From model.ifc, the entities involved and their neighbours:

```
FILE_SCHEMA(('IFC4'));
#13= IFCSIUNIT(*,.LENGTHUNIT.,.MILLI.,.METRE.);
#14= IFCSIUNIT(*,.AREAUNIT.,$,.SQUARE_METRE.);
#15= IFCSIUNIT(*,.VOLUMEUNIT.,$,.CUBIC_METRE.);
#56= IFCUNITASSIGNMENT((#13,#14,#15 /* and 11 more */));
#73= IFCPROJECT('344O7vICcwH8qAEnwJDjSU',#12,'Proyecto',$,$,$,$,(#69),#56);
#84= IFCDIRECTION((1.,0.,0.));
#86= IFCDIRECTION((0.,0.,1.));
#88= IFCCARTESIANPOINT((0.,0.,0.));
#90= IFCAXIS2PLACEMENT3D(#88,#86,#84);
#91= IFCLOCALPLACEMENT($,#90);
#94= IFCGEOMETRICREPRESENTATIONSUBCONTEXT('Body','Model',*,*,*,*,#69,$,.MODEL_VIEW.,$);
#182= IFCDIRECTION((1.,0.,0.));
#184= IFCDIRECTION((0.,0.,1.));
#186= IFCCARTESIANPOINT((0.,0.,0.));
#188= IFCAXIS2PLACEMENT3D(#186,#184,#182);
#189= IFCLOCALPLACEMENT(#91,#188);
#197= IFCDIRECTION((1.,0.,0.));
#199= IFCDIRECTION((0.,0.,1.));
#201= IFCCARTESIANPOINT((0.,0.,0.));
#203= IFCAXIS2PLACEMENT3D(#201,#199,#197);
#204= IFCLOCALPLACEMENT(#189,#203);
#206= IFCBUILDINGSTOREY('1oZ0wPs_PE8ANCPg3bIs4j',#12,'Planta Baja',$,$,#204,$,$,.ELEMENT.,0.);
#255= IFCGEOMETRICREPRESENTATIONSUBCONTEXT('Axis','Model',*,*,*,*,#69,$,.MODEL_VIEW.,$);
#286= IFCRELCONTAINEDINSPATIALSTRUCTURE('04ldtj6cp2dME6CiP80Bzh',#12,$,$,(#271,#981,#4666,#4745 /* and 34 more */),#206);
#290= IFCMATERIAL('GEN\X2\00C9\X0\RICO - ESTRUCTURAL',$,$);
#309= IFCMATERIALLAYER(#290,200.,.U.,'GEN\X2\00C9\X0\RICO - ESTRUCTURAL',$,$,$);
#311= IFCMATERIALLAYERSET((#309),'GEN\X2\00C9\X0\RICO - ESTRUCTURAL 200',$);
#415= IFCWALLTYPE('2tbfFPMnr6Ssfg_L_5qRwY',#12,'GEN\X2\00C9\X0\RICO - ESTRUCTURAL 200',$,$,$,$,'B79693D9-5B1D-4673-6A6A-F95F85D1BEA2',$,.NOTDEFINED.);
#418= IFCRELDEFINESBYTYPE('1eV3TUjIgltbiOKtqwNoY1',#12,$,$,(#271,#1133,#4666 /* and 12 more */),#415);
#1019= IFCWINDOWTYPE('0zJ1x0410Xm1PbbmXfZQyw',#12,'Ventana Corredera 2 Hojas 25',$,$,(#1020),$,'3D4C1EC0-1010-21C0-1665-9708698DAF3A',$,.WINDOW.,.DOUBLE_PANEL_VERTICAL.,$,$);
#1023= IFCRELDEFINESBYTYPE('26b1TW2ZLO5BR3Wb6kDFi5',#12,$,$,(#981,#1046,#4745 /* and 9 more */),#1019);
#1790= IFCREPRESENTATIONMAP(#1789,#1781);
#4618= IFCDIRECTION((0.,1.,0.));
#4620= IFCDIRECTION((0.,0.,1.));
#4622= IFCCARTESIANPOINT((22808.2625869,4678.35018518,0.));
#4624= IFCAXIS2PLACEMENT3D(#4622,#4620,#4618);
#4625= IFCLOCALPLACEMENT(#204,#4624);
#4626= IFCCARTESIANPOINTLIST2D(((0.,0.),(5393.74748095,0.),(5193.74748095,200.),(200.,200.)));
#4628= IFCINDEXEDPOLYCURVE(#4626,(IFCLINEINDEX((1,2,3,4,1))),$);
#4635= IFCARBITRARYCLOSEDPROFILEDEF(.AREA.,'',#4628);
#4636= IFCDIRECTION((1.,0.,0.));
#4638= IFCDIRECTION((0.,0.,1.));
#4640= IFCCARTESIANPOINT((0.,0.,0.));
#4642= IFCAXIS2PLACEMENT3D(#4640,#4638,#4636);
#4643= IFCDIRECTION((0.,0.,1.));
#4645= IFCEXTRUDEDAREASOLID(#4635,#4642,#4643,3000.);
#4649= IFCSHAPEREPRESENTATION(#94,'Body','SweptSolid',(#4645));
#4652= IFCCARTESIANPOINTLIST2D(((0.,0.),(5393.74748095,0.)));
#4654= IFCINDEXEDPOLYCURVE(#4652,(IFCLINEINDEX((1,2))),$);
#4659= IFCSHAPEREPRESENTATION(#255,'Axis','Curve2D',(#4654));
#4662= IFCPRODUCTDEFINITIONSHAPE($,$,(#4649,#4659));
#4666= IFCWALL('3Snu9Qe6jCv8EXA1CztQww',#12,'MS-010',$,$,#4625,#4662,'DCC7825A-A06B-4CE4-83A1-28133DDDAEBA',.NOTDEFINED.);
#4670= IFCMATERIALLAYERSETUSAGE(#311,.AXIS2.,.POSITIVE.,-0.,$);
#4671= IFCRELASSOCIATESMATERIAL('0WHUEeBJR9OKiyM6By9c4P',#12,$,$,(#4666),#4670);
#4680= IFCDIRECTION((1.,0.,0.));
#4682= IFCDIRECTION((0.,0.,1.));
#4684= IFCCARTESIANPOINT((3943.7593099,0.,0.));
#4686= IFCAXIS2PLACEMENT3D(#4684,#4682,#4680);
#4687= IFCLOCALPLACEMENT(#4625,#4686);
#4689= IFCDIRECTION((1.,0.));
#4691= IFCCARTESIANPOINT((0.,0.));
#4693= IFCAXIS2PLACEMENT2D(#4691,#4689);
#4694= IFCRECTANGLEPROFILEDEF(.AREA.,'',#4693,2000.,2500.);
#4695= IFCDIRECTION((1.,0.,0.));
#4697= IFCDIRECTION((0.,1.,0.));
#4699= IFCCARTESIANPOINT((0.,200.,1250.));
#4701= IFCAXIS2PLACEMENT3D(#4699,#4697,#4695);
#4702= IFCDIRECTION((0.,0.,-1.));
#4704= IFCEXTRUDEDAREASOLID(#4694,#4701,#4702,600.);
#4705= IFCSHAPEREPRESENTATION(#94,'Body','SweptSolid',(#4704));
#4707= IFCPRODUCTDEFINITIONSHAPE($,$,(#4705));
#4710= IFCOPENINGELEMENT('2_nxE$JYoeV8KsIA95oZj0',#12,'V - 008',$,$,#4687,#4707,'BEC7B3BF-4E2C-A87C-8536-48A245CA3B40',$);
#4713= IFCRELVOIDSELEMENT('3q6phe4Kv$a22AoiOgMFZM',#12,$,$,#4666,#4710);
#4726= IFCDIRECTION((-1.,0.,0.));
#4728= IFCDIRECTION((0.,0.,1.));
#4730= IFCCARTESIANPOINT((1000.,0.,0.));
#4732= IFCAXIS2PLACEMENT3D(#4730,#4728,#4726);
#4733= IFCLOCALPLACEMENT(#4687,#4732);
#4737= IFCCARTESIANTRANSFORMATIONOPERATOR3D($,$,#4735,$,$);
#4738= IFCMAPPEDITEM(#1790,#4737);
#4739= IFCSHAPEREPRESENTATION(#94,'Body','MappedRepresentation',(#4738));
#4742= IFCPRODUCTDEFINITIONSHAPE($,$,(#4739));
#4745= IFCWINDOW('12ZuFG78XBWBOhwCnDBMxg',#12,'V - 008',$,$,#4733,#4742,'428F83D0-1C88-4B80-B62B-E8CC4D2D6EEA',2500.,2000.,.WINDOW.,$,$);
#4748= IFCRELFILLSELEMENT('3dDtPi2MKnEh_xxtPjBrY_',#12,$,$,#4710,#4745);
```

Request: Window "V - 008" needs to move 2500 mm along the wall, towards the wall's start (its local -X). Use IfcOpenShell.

```python
import ifcopenshell
import ifcopenshell.api.geometry
import ifcopenshell.util.placement

model = ifcopenshell.open("model.ifc")

window = model.by_guid("12ZuFG78XBWBOhwCnDBMxg")
opening = window.FillsVoids[0].RelatingOpeningElement
wall = opening.VoidsElements[0].RelatingBuildingElement

wall_matrix = ifcopenshell.util.placement.get_local_placement(wall.ObjectPlacement)
shift = wall_matrix[:3, 0] * -2500.0
before = ifcopenshell.util.placement.get_local_placement(window.ObjectPlacement)[:3, 3].copy()

# The window is placed relative to its opening, so it follows when the opening moves.
matrix = ifcopenshell.util.placement.get_local_placement(opening.ObjectPlacement)
matrix[:3, 3] += shift
ifcopenshell.api.geometry.edit_object_placement(
    model, product=opening, matrix=matrix, is_si=False, should_transform_children=True
)

after = ifcopenshell.util.placement.get_local_placement(window.ObjectPlacement)[:3, 3]
print("window moved by", (after - before).round(3) + 0.0)

model.write("model-out.ifc")
```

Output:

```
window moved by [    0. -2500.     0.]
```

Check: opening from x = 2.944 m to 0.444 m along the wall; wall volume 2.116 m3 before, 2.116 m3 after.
